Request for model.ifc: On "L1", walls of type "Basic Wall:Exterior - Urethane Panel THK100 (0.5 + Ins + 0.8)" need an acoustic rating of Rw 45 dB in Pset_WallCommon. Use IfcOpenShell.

First a look at what the model holds.

```python
import ifcopenshell
import ifcopenshell.util.element

model = ifcopenshell.open("model.ifc")
print(model.schema)
storey = next(s for s in model.by_type("IfcBuildingStorey") if s.Name == "L1")
walls = [e for e in ifcopenshell.util.element.get_decomposition(storey) if e.is_a("IfcWall")]
seen = {}
for e in walls:
    element_type = ifcopenshell.util.element.get_type(e)
    key = (element_type.Name if element_type != e and element_type else None, ifcopenshell.util.element.get_pset(e, "Pset_WallCommon", "AcousticRating"))
    seen[key] = seen.get(key, 0) + 1
for (name, value), count in sorted(seen.items(), key=str):
    print(count, "x", name, "|", value)
```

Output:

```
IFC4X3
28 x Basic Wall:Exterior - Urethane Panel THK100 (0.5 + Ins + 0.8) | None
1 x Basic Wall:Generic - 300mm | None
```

```python
import ifcopenshell
import ifcopenshell.api.pset
import ifcopenshell.util.element

model = ifcopenshell.open("model.ifc")

storey = next(s for s in model.by_type("IfcBuildingStorey") if s.Name == "L1")
walls = [e for e in ifcopenshell.util.element.get_decomposition(storey) if e.is_a("IfcWall")]

count = 0
for e in walls:
    element_type = ifcopenshell.util.element.get_type(e)
    if element_type in (None, e) or element_type.Name != "Basic Wall:Exterior - Urethane Panel THK100 (0.5 + Ins + 0.8)":
        continue
    # add_pset returns the element's existing set when there is one.
    pset = ifcopenshell.api.pset.add_pset(model, product=e, name="Pset_WallCommon")
    ifcopenshell.api.pset.edit_pset(model, pset=pset, properties={"AcousticRating": "Rw 45 dB"})
    count += 1

print(count, "walls updated")

model.write("model_rev.ifc")
```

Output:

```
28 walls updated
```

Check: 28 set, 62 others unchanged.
